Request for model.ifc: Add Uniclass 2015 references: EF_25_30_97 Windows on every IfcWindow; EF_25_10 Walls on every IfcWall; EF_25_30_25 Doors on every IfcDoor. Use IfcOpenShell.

First a look at what the model holds.

```python
import ifcopenshell

model = ifcopenshell.open("model.ifc")
print(model.schema)
print("classifications:", [c.Name for c in model.by_type("IfcClassification")])
for ifc_class in ("IfcDoor", "IfcRoof", "IfcStair", "IfcWall", "IfcWindow"):
    print(ifc_class, len(model.by_type(ifc_class)))
```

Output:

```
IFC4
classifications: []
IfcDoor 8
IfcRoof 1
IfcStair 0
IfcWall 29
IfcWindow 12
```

```python
import ifcopenshell
import ifcopenshell.api.classification

model = ifcopenshell.open("model.ifc")

system = ifcopenshell.api.classification.add_classification(model, classification="Uniclass 2015")

codes = {
    "IfcWindow": ("EF_25_30_97", "Windows"),
    "IfcWall": ("EF_25_10", "Walls"),
    "IfcDoor": ("EF_25_30_25", "Doors"),
}
for ifc_class, (code, name) in codes.items():
    products = model.by_type(ifc_class)
    ifcopenshell.api.classification.add_reference(
        model, products=products, classification=system, identification=code, name=name
    )
    print(code, len(products))

model.write("model_edited.ifc")
```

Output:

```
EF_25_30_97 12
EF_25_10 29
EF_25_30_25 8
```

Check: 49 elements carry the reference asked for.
